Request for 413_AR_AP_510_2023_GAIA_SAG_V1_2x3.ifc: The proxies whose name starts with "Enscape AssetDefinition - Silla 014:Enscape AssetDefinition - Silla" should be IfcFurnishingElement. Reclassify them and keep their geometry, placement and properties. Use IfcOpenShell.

First a look at what the model holds.

```python
import re

import ifcopenshell

model = ifcopenshell.open("413_AR_AP_510_2023_GAIA_SAG_V1_2x3.ifc")
print(model.schema)
seen = {}
for e in model.by_type("IfcBuildingElementProxy"):
    name = re.sub(r":\d+(:\d+)?$", "", e.Name or "")  # drop the element id that some exporters append
    seen[name] = seen.get(name, 0) + 1
for name, count in sorted(seen.items()):
    print(count, "x", name)
```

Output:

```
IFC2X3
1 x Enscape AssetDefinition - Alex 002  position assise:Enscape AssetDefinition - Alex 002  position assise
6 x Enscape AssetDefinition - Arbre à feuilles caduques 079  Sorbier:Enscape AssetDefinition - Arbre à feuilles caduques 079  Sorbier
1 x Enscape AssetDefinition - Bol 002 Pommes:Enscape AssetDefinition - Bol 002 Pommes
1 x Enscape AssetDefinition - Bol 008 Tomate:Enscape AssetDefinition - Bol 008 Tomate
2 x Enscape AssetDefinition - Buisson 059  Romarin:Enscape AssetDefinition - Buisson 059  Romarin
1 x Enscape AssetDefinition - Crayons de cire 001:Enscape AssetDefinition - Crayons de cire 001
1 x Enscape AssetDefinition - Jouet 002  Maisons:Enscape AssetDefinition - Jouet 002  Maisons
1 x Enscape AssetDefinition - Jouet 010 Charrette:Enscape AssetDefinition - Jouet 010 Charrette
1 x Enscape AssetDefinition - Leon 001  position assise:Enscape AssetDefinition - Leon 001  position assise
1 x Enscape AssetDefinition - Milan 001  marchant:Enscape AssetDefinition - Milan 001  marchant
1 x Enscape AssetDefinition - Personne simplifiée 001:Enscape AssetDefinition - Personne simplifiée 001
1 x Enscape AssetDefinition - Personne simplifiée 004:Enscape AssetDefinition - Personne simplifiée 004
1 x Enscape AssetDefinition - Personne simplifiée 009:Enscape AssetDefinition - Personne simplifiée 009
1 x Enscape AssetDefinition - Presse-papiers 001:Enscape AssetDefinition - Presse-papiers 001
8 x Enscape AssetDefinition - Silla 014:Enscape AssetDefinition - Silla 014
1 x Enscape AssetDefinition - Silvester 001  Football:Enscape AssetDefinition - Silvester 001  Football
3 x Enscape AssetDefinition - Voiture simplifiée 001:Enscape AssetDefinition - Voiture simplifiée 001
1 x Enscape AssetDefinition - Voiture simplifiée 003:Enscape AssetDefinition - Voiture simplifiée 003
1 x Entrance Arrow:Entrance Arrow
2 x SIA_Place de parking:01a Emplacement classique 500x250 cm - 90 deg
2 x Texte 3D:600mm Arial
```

```python
import ifcopenshell
import ifcopenshell.api.root

model = ifcopenshell.open("413_AR_AP_510_2023_GAIA_SAG_V1_2x3.ifc")

proxies = [e.id() for e in model.by_type("IfcBuildingElementProxy") if (e.Name or "").startswith("Enscape AssetDefinition - Silla 014:Enscape AssetDefinition - Silla")]
for step_id in proxies:
    proxy = model.by_id(step_id)
    # Reclassifying a typed element also reclassifies its type and the type's other occurrences.
    if proxy.is_a("IfcBuildingElementProxy"):
        ifcopenshell.api.root.reassign_class(model, product=proxy, ifc_class="IfcFurnishingElement")

print(sum(model.by_id(i).is_a("IfcFurnishingElement") for i in proxies), "reclassified")

model.write("413_AR_AP_510_2023_GAIA_SAG_V1_2x3_rev.ifc")
```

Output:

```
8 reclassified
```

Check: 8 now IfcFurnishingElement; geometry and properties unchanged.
